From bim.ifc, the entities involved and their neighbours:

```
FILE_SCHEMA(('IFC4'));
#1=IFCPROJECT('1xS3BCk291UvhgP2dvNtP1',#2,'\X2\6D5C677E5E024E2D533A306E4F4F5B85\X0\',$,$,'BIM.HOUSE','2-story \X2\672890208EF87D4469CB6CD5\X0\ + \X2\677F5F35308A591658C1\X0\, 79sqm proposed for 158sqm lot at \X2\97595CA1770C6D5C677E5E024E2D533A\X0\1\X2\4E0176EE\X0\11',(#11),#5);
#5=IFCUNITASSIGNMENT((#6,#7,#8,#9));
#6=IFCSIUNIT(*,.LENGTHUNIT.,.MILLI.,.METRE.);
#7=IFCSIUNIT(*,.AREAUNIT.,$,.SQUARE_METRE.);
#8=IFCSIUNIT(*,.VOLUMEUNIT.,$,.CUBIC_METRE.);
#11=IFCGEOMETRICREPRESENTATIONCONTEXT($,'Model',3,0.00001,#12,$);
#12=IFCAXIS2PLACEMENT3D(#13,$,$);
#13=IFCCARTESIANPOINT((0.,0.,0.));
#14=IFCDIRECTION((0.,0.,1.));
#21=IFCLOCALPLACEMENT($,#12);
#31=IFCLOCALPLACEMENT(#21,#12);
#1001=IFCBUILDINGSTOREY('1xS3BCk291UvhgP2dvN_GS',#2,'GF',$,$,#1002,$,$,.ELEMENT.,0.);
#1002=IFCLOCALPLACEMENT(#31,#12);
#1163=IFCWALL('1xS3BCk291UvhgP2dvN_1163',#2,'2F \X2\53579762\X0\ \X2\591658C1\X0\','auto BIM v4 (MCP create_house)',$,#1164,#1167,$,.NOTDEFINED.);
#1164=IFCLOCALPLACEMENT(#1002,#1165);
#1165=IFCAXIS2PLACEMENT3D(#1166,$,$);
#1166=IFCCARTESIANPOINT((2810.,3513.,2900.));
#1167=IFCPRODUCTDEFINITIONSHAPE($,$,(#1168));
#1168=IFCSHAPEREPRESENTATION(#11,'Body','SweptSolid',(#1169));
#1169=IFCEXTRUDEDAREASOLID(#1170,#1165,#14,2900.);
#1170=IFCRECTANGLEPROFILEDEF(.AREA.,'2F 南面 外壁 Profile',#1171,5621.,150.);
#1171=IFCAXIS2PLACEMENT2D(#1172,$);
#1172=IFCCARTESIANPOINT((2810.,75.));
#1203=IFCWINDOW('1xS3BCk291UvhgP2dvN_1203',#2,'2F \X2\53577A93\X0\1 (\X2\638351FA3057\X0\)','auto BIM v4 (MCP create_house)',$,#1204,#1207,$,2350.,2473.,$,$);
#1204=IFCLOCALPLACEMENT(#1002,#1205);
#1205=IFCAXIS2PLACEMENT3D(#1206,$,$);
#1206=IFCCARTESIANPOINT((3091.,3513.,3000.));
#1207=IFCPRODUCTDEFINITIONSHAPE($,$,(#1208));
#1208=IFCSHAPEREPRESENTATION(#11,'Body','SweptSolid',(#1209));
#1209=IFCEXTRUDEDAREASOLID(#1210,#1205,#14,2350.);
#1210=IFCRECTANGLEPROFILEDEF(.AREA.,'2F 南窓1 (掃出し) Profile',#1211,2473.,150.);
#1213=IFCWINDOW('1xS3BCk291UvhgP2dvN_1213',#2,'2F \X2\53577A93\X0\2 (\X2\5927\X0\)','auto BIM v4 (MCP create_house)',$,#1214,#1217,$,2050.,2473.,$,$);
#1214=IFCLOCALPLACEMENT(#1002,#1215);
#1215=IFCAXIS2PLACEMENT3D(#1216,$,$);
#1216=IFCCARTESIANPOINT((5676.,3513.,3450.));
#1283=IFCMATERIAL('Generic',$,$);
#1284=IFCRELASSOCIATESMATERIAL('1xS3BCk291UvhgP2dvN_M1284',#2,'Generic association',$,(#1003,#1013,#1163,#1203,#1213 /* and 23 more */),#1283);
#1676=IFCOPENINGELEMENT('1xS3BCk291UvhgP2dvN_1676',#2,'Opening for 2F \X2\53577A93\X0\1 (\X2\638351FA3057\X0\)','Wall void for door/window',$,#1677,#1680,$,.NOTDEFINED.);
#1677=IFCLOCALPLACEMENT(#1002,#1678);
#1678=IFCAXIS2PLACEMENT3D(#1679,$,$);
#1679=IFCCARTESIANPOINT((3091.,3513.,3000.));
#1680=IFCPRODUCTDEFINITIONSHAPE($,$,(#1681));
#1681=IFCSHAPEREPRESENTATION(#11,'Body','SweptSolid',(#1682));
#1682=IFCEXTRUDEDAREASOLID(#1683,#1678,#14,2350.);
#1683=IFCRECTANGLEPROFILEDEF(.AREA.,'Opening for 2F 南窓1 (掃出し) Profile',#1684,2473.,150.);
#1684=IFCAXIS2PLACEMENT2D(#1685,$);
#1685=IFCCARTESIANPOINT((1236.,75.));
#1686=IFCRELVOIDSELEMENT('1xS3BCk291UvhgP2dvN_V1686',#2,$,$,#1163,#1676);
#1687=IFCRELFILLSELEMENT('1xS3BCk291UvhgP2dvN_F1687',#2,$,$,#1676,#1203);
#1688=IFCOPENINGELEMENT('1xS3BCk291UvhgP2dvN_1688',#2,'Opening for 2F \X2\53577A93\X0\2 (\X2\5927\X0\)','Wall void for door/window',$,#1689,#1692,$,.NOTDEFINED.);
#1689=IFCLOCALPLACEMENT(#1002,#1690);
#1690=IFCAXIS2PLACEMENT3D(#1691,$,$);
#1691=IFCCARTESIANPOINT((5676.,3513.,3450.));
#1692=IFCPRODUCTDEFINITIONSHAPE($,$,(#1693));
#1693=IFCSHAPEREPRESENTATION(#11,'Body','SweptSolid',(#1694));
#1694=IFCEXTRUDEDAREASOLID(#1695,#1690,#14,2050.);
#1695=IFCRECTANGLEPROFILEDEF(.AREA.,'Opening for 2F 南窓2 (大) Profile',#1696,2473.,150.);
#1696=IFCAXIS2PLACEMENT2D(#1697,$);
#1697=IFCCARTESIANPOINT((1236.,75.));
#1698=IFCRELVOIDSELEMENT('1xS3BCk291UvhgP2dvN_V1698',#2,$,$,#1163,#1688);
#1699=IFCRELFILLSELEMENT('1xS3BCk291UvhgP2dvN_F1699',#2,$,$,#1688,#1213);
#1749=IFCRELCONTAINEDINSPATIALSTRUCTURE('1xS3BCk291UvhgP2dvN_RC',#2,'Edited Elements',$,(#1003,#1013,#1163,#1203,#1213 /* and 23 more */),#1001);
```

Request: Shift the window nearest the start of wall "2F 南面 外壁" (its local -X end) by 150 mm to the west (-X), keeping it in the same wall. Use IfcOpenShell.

```python
import ifcopenshell
import ifcopenshell.api.geometry
import ifcopenshell.util.placement

model = ifcopenshell.open("bim.ifc")

window = model.by_guid("1xS3BCk291UvhgP2dvN_1203")
opening = window.FillsVoids[0].RelatingOpeningElement
wall = opening.VoidsElements[0].RelatingBuildingElement

wall_matrix = ifcopenshell.util.placement.get_local_placement(wall.ObjectPlacement)
shift = wall_matrix[:3, 0] * -150.0
before = ifcopenshell.util.placement.get_local_placement(window.ObjectPlacement)[:3, 3].copy()

# The window is not placed relative to its opening, so move both.
for product in (opening, window):
    matrix = ifcopenshell.util.placement.get_local_placement(product.ObjectPlacement)
    matrix[:3, 3] += shift
    ifcopenshell.api.geometry.edit_object_placement(model, product=product, matrix=matrix, is_si=False)

after = ifcopenshell.util.placement.get_local_placement(window.ObjectPlacement)[:3, 3]
print("window moved by", (after - before).round(3) + 0.0)

model.write("bim_v2.ifc")
```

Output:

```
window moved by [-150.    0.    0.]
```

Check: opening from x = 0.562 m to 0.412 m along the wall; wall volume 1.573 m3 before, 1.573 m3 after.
